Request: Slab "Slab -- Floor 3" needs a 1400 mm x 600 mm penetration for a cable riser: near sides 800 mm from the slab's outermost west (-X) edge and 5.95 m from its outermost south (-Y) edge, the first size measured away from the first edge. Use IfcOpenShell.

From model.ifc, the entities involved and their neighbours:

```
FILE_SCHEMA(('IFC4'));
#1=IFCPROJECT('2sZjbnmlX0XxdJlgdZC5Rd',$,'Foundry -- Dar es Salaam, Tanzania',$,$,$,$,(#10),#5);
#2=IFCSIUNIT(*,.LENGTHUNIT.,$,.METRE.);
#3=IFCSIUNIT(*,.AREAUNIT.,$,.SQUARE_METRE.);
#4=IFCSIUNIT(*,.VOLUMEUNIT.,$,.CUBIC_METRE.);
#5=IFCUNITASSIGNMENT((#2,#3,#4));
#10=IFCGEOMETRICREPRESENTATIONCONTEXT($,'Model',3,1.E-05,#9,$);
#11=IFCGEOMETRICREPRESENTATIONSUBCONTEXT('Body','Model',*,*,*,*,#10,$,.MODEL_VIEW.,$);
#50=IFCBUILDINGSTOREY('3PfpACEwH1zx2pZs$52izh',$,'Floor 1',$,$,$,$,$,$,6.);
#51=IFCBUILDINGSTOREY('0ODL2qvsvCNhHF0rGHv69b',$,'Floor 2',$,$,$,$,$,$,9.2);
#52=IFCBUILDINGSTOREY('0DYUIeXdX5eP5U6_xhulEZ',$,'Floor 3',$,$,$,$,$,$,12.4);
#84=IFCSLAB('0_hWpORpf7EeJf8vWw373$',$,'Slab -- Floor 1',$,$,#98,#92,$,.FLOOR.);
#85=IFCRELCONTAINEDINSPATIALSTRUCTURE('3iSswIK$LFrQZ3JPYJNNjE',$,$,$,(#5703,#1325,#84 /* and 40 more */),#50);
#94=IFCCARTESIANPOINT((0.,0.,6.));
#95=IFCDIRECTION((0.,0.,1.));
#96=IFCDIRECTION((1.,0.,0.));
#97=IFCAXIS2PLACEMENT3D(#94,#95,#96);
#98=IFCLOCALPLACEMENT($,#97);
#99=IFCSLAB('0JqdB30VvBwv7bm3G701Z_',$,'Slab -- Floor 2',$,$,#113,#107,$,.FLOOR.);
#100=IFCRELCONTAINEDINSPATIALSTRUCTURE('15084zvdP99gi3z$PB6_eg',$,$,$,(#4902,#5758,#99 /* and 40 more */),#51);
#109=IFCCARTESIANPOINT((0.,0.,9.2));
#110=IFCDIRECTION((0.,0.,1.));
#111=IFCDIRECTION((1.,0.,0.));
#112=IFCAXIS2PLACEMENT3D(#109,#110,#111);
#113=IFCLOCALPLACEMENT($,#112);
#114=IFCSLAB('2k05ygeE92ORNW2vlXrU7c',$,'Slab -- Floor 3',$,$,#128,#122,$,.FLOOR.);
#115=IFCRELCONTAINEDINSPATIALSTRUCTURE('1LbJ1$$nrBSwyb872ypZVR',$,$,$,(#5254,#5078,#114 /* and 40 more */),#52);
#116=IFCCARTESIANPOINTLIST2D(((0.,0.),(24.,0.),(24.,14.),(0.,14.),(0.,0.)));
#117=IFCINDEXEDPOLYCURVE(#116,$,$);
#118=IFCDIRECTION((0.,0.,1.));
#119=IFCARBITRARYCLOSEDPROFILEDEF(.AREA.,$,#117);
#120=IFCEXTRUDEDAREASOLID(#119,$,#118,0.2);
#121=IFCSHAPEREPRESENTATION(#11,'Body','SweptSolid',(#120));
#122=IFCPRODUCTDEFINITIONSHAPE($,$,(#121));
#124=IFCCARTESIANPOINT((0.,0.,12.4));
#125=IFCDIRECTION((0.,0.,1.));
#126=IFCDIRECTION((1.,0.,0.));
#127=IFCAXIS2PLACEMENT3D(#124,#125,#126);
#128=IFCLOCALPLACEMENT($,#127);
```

```python
import numpy as np
import ifcopenshell
import ifcopenshell.api.feature
import ifcopenshell.api.geometry
import ifcopenshell.api.root
import ifcopenshell.geom
import ifcopenshell.util.placement
import ifcopenshell.util.representation
import ifcopenshell.util.shape
import ifcopenshell.util.unit

model = ifcopenshell.open("model.ifc")
unit_scale = ifcopenshell.util.unit.calculate_unit_scale(model)
settings = ifcopenshell.geom.settings()


def volume(element):
    """Net volume in cubic metres, openings subtracted."""
    shape = ifcopenshell.geom.create_shape(settings, element)
    return ifcopenshell.util.shape.get_volume(shape.geometry)


slab = model.by_id(114)
before = volume(slab)

# Extent in the slab's own axes, in metres. The edges named are its -X and -Y sides.
slab_shape = ifcopenshell.geom.create_shape(settings, slab)
vertices = ifcopenshell.util.shape.get_vertices(slab_shape.geometry)
x_min, y_min, bottom = vertices.min(axis=0)
top = vertices[:, 2].max()

opening = ifcopenshell.api.root.create_entity(model, ifc_class="IfcOpeningElement", name="Cable riser opening", predefined_type="OPENING")
context = ifcopenshell.util.representation.get_context(model, "Model", "Body", "MODEL_VIEW")
width, depth = 1.4, 0.6
outline = [(0.0, 0.0), (width, 0.0), (width, depth), (0.0, depth), (0.0, 0.0)]
# Overshoot both faces by 50 mm so the cut is clean.
shape = ifcopenshell.api.geometry.add_slab_representation(
    model, context=context, depth=top - bottom + 0.1, polyline=outline
)
ifcopenshell.api.geometry.assign_representation(model, product=opening, representation=shape)

matrix = ifcopenshell.util.placement.get_local_placement(slab.ObjectPlacement)
matrix[:, 3] = matrix @ np.append(np.array([x_min + 0.8, y_min + 5.95, bottom - 0.05]) / unit_scale, 1.0)
ifcopenshell.api.geometry.edit_object_placement(model, product=opening, matrix=matrix, is_si=False)
ifcopenshell.api.feature.add_feature(model, feature=opening, element=slab)

after = volume(slab)

print(f"slab volume {before:.3f} -> {after:.3f} m3")

model.write("model-out.ifc")
```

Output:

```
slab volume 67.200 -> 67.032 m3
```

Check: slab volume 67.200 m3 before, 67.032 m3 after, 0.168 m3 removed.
